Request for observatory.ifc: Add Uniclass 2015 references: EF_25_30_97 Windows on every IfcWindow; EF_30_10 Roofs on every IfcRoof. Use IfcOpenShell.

First a look at what the model holds.

```python
import ifcopenshell

model = ifcopenshell.open("observatory.ifc")
print(model.schema)
print("classifications:", [c.Name for c in model.by_type("IfcClassification")])
for ifc_class in ("IfcDoor", "IfcRoof", "IfcStair", "IfcWall", "IfcWindow"):
    print(ifc_class, len(model.by_type(ifc_class)))
```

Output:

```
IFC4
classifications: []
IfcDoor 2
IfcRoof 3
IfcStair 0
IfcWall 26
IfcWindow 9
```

```python
import ifcopenshell
import ifcopenshell.api.classification

model = ifcopenshell.open("observatory.ifc")

system = ifcopenshell.api.classification.add_classification(model, classification="Uniclass 2015")

codes = {
    "IfcWindow": ("EF_25_30_97", "Windows"),
    "IfcRoof": ("EF_30_10", "Roofs"),
}
for ifc_class, (code, name) in codes.items():
    products = model.by_type(ifc_class)
    ifcopenshell.api.classification.add_reference(
        model, products=products, classification=system, identification=code, name=name
    )
    print(code, len(products))

model.write("observatory_edited.ifc")
```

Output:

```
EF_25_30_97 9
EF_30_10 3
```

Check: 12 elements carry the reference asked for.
